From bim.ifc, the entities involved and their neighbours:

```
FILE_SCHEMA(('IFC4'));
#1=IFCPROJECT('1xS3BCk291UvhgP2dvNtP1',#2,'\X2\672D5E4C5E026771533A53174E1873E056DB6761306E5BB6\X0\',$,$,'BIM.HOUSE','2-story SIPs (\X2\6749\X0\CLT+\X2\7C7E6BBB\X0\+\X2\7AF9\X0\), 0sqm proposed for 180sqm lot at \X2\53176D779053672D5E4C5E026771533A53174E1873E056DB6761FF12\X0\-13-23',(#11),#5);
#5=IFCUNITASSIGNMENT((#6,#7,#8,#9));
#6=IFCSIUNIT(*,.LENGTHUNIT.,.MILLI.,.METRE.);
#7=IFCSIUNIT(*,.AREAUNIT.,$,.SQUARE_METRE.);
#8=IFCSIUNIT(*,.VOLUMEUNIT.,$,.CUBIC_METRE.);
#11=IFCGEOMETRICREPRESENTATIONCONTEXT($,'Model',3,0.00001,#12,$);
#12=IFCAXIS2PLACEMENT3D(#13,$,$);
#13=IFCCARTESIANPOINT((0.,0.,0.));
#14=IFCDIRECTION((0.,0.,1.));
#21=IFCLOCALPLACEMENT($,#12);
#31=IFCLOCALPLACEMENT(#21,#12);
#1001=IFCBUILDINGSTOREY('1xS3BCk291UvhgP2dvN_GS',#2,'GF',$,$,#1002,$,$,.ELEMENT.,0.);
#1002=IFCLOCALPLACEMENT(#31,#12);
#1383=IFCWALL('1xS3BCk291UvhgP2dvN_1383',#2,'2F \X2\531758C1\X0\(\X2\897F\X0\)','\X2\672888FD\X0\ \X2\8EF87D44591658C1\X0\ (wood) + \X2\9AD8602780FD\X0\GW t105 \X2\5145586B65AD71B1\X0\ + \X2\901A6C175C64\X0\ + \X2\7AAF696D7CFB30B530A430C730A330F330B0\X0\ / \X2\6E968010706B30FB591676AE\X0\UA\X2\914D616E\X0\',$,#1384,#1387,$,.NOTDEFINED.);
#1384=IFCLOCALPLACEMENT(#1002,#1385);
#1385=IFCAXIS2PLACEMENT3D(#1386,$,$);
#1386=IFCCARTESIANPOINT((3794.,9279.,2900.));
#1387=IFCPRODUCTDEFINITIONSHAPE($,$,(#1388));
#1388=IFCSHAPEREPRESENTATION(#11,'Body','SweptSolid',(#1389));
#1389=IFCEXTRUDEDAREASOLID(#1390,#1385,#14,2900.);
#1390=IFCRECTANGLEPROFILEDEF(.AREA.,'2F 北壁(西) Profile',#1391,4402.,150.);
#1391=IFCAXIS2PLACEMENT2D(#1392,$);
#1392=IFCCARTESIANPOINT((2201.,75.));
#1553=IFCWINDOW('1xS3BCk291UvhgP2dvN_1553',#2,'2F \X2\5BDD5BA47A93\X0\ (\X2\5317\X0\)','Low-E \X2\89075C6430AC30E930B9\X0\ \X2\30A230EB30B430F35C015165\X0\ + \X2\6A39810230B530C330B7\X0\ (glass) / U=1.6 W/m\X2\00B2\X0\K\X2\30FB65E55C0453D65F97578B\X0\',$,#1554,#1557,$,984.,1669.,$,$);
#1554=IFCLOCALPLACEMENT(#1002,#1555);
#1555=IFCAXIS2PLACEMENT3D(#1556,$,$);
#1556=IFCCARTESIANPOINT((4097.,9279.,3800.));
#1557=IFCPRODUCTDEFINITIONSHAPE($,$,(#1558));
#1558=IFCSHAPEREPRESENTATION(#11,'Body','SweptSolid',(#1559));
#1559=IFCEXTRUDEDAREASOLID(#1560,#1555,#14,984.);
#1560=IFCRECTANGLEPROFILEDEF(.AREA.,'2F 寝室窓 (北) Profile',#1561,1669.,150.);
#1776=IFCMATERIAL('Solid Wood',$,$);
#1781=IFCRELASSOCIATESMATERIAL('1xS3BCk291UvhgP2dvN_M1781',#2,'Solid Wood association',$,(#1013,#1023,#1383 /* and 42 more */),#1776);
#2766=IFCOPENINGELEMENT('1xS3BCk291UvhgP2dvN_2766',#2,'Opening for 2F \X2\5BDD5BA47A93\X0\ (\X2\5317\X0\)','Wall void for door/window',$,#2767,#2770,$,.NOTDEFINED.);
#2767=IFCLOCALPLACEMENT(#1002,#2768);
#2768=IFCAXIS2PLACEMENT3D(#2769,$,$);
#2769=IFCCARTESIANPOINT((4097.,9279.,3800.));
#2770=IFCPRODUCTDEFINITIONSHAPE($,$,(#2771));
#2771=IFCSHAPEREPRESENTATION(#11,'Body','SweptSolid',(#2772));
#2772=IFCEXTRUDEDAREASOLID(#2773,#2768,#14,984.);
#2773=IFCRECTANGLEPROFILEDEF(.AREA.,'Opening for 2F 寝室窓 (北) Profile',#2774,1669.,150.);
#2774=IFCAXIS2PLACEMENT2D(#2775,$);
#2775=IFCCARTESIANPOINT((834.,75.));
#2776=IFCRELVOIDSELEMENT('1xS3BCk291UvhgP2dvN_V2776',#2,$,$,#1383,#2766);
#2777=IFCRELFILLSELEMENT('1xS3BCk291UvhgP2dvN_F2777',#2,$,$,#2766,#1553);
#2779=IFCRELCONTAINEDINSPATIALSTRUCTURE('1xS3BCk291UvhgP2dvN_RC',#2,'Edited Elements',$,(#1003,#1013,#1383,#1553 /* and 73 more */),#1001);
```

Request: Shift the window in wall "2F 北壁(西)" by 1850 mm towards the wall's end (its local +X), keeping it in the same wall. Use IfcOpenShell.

```python
import ifcopenshell
import ifcopenshell.api.geometry
import ifcopenshell.util.placement
import ifcopenshell.util.unit

model = ifcopenshell.open("bim.ifc")
unit_scale = ifcopenshell.util.unit.calculate_unit_scale(model)

window = model.by_guid("1xS3BCk291UvhgP2dvN_1553")
opening = window.FillsVoids[0].RelatingOpeningElement
wall = opening.VoidsElements[0].RelatingBuildingElement

wall_matrix = ifcopenshell.util.placement.get_local_placement(wall.ObjectPlacement)
shift = wall_matrix[:3, 0] * 1.85 / unit_scale
before = ifcopenshell.util.placement.get_local_placement(window.ObjectPlacement)[:3, 3].copy()

# The window is not placed relative to its opening, so move both.
for product in (opening, window):
    matrix = ifcopenshell.util.placement.get_local_placement(product.ObjectPlacement)
    matrix[:3, 3] += shift
    ifcopenshell.api.geometry.edit_object_placement(model, product=product, matrix=matrix, is_si=False)

after = ifcopenshell.util.placement.get_local_placement(window.ObjectPlacement)[:3, 3]
print("window moved by", (after - before).round(3) + 0.0)

model.write("bim-out.ifc")
```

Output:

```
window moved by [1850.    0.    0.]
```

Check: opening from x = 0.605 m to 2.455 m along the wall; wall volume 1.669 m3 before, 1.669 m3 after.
